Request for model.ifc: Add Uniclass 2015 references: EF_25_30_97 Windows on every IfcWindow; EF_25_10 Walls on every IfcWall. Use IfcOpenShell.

First a look at what the model holds.

```python
import ifcopenshell

model = ifcopenshell.open("model.ifc")
print(model.schema)
print("classifications:", [c.Name for c in model.by_type("IfcClassification")])
for ifc_class in ("IfcDoor", "IfcRoof", "IfcStair", "IfcWall", "IfcWindow"):
    print(ifc_class, len(model.by_type(ifc_class)))
```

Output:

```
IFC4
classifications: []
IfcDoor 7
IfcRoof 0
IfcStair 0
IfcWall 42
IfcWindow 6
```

```python
import ifcopenshell
import ifcopenshell.api.classification

model = ifcopenshell.open("model.ifc")

system = ifcopenshell.api.classification.add_classification(model, classification="Uniclass 2015")

codes = {
    "IfcWindow": ("EF_25_30_97", "Windows"),
    "IfcWall": ("EF_25_10", "Walls"),
}
for ifc_class, (code, name) in codes.items():
    products = model.by_type(ifc_class)
    ifcopenshell.api.classification.add_reference(
        model, products=products, classification=system, identification=code, name=name
    )
    print(code, len(products))

model.write("model_edited.ifc")
```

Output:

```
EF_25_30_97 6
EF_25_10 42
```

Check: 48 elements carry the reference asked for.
